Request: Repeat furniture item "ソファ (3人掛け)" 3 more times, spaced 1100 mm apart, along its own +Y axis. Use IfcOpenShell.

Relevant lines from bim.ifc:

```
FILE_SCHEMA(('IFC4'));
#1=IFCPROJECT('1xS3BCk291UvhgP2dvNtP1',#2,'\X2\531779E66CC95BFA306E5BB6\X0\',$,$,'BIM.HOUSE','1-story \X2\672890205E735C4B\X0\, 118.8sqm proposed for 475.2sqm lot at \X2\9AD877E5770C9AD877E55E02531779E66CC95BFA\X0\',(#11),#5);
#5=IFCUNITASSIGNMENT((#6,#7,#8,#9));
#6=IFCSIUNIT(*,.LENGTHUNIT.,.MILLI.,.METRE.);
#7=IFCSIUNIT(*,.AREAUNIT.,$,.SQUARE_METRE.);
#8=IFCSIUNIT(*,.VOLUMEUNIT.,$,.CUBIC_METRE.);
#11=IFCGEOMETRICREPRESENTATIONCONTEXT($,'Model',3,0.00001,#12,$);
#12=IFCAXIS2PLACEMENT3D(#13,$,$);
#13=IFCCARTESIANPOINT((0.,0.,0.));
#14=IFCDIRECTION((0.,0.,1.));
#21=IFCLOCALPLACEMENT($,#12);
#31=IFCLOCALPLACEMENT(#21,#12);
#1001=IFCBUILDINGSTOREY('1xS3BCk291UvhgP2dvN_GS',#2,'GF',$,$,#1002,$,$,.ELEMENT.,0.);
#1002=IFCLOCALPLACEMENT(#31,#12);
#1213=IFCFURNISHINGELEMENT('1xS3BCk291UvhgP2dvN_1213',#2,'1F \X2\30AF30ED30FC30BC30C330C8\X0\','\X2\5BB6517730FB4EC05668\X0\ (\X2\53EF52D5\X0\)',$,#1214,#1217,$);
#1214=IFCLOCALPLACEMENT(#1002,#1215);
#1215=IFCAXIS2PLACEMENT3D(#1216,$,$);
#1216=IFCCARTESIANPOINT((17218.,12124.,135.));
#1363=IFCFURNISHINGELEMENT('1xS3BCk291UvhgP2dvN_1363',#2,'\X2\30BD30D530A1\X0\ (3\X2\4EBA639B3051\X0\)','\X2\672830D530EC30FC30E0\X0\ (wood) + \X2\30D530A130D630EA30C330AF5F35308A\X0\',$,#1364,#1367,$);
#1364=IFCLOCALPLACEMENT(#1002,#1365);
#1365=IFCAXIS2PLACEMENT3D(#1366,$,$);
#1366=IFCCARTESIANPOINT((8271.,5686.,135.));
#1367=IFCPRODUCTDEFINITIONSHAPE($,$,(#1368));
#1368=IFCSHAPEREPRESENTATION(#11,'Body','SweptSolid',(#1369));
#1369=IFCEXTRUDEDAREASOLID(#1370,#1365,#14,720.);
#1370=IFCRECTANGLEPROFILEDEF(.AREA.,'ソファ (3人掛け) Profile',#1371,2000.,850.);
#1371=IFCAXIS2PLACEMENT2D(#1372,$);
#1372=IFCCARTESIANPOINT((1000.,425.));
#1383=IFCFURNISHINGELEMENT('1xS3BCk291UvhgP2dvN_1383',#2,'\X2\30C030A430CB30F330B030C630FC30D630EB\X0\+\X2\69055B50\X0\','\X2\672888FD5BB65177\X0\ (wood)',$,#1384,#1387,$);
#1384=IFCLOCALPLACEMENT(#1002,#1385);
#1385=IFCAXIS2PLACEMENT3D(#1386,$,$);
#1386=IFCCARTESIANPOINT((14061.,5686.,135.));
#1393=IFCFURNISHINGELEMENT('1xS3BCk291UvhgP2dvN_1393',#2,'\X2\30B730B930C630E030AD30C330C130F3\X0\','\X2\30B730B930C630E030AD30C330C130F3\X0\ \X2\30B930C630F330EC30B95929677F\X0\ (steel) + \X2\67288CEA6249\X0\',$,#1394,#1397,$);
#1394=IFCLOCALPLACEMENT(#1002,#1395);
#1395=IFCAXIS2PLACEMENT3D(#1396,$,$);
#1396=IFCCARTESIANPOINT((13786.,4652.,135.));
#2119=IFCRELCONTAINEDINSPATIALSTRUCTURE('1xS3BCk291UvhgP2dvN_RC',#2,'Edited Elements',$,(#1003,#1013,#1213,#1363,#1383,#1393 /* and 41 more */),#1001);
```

```python
import ifcopenshell
import ifcopenshell.api.geometry
import ifcopenshell.api.root
import ifcopenshell.util.element
import ifcopenshell.util.placement

model = ifcopenshell.open("bim.ifc")


def reuse_history(source, copy):
    """copy_class also copies each property set's owner history, people and application; keep the originals."""
    for rel in copy.IsDefinedBy:
        if rel.is_a("IfcRelDefinesByProperties") and (history := rel.RelatingPropertyDefinition.OwnerHistory):
            rel.RelatingPropertyDefinition.OwnerHistory = source.OwnerHistory
            ifcopenshell.util.element.remove_deep2(model, history)


source = model.by_guid("1xS3BCk291UvhgP2dvN_1363")
base = ifcopenshell.util.placement.get_local_placement(source.ObjectPlacement)
step = base[:3, 1] * 1100.0

for i in range(1, 4):
    copy = ifcopenshell.api.root.copy_class(model, product=source)
    copy.Representation = ifcopenshell.util.element.copy_deep(
        model, source.Representation, exclude=["IfcGeometricRepresentationContext", "IfcRepresentationMap"]
    )
    reuse_history(source, copy)
    matrix = base.copy()
    matrix[:3, 3] += i * step
    print("added at", matrix[:3, 3].round(3) + 0.0)
    ifcopenshell.api.geometry.edit_object_placement(model, product=copy, matrix=matrix, is_si=False)

model.write("bim_updated.ifc")
```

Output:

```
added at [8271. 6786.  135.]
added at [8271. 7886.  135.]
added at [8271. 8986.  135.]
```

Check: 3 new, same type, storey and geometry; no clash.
